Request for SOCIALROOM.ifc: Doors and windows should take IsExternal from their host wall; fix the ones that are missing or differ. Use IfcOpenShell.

First a look at what the model holds.

```python
import ifcopenshell
import ifcopenshell.util.element

model = ifcopenshell.open("SOCIALROOM.ifc")
print(model.schema)
seen = {}
for e in model.by_type("IfcDoor") + model.by_type("IfcWindow"):
    if not e.FillsVoids:
        continue
    host = e.FillsVoids[0].RelatingOpeningElement.VoidsElements[0].RelatingBuildingElement
    own = ifcopenshell.util.element.get_pset(e, f"Pset_{e.is_a()[3:].removesuffix('StandardCase')}Common", "IsExternal")
    wall = ifcopenshell.util.element.get_pset(host, "Pset_WallCommon", "IsExternal")
    seen[e.is_a(), own, wall] = seen.get((e.is_a(), own, wall), 0) + 1
for (cls, own, wall), count in sorted(seen.items(), key=str):
    print(count, cls, "IsExternal:", own, "| host wall:", wall)
```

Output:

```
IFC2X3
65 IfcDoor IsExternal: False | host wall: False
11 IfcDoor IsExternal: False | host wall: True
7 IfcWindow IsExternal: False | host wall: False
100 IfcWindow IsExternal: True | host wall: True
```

```python
import ifcopenshell
import ifcopenshell.api.pset
import ifcopenshell.util.element

model = ifcopenshell.open("SOCIALROOM.ifc")

count = 0
for ifc_class, pset_name in (("IfcDoor", "Pset_DoorCommon"), ("IfcWindow", "Pset_WindowCommon")):
    for e in model.by_type(ifc_class):
        if not e.FillsVoids:
            continue
        host = e.FillsVoids[0].RelatingOpeningElement.VoidsElements[0].RelatingBuildingElement
        external = ifcopenshell.util.element.get_pset(host, "Pset_WallCommon", "IsExternal")
        if external is None or ifcopenshell.util.element.get_pset(e, pset_name, "IsExternal") == external:
            continue
        pset = ifcopenshell.api.pset.add_pset(model, product=e, name=pset_name)
        ifcopenshell.api.pset.edit_pset(model, pset=pset, properties={"IsExternal": external})
        count += 1

print(count, "updated")

model.write("SOCIALROOM_v2.ifc")
```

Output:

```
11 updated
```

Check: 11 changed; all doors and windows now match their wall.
